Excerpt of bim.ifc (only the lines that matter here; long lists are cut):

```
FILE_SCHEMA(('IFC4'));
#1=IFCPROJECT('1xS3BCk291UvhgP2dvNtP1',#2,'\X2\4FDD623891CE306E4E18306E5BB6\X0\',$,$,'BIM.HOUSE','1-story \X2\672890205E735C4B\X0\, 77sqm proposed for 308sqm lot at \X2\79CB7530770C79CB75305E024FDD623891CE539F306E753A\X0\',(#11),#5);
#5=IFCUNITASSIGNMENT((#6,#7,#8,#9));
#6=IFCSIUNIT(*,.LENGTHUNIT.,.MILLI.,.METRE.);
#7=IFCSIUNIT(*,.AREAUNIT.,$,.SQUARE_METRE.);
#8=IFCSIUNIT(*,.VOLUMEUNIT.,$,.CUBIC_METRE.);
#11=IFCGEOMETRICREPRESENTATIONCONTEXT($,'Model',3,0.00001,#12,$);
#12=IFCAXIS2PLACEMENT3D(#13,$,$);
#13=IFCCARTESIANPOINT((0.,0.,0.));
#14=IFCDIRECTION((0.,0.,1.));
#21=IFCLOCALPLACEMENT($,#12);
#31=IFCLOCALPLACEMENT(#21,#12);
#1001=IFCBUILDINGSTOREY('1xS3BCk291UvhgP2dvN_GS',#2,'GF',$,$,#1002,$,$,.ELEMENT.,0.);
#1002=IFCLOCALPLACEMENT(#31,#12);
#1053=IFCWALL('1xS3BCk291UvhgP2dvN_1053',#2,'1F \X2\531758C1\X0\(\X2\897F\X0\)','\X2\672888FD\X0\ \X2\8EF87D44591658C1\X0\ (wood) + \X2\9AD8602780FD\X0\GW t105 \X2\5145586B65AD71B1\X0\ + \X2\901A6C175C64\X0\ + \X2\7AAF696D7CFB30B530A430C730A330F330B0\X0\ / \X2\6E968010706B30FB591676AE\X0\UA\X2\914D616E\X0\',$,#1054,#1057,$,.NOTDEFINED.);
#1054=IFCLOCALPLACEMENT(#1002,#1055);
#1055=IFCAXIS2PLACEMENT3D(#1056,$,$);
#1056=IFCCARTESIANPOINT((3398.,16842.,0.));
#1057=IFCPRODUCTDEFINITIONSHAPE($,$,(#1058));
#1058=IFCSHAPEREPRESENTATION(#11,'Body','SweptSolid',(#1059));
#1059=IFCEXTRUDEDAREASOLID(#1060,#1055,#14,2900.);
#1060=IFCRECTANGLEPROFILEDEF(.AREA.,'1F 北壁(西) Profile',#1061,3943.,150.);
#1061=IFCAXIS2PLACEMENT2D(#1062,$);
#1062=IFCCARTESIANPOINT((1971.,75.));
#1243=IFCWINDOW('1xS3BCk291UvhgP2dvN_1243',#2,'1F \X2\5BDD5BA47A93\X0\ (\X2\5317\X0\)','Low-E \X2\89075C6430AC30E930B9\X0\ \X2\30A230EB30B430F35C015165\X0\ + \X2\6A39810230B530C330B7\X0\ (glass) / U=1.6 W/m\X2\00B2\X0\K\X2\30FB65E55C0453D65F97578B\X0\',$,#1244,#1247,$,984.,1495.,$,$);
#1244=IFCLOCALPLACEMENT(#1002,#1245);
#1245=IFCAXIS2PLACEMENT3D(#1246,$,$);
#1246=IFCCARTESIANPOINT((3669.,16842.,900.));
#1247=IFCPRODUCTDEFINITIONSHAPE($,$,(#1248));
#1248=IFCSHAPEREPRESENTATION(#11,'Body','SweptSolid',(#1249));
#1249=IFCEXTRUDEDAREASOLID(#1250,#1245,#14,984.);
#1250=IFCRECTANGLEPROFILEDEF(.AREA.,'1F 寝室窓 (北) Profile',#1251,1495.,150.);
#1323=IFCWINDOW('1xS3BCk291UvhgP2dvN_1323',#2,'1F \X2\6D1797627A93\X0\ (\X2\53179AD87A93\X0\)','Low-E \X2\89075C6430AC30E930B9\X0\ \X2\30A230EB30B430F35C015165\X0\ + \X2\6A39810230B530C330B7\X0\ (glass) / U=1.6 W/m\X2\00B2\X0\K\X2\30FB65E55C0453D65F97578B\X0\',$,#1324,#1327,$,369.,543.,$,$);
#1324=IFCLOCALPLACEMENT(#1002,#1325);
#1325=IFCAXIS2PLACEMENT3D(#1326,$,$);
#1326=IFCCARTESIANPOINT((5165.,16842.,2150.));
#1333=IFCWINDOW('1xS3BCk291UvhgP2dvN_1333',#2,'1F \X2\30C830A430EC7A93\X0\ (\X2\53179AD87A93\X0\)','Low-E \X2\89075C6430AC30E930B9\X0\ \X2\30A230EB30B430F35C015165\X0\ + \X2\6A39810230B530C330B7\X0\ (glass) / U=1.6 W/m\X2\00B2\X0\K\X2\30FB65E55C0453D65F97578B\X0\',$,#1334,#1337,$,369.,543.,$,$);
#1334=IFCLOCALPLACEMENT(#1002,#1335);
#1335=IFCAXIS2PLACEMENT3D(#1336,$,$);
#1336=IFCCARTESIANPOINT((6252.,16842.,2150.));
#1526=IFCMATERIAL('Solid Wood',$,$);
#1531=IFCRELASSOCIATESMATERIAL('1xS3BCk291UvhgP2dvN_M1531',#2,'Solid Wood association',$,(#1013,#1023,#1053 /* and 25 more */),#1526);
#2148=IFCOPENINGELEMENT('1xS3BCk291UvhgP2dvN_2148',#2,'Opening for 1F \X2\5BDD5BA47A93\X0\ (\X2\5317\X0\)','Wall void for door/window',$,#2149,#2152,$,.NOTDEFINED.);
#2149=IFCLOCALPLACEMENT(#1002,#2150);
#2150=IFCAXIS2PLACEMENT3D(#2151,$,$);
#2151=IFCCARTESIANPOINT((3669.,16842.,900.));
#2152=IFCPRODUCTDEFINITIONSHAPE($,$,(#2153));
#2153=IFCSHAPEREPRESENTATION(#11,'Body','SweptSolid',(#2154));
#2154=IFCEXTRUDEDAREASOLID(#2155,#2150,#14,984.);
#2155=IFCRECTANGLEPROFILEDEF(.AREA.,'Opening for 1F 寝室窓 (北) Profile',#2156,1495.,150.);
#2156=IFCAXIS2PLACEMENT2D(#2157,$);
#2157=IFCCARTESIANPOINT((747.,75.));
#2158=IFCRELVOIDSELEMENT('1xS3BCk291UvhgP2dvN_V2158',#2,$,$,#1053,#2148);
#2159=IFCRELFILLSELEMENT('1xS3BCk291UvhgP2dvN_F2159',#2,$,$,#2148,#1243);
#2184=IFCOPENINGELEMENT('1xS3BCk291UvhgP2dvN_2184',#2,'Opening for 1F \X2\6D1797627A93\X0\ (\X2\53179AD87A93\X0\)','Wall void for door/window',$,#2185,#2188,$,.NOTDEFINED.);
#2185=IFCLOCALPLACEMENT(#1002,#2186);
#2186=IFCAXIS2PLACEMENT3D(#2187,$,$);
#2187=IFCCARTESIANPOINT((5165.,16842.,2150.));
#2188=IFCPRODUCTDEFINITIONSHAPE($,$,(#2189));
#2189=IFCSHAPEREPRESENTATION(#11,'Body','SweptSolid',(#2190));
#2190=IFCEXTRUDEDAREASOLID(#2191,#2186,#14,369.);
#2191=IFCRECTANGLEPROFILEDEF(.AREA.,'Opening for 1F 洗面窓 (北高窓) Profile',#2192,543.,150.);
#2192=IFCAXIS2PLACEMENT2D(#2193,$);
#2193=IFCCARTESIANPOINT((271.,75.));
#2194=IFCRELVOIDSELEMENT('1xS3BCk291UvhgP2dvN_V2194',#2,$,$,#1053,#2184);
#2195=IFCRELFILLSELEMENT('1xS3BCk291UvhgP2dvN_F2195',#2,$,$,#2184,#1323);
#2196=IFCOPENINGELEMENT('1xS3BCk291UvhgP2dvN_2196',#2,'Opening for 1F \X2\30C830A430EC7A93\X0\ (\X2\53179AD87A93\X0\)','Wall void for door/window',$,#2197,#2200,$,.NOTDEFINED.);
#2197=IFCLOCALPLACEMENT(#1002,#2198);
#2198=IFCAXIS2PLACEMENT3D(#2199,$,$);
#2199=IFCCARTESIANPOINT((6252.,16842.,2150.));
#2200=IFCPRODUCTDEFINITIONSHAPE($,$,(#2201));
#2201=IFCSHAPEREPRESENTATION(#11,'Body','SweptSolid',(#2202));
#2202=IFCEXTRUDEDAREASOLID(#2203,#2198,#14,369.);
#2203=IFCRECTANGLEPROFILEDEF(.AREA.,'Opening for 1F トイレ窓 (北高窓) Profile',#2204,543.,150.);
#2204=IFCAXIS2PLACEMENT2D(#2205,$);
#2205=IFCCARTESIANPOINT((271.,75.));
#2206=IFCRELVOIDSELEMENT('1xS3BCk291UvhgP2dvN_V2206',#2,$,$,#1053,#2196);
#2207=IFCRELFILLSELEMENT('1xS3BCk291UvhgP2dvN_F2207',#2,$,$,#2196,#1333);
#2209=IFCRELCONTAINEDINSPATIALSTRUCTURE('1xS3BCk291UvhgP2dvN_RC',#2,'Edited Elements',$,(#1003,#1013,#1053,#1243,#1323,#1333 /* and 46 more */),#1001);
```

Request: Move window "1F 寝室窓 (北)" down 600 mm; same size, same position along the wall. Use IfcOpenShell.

```python
import numpy as np
import ifcopenshell
import ifcopenshell.api.geometry
import ifcopenshell.util.placement
import ifcopenshell.util.unit

model = ifcopenshell.open("bim.ifc")
unit_scale = ifcopenshell.util.unit.calculate_unit_scale(model)

window = model.by_guid("1xS3BCk291UvhgP2dvN_1243")
opening = window.FillsVoids[0].RelatingOpeningElement
dz = -600.0

shift = np.array([0.0, 0.0, dz])
# The window is not placed relative to its opening, so move both.
for product in (opening, window):
    matrix = ifcopenshell.util.placement.get_local_placement(product.ObjectPlacement)
    matrix[:3, 3] += shift
    ifcopenshell.api.geometry.edit_object_placement(model, product=product, matrix=matrix, is_si=False)

print(f"moved by {dz * unit_scale:+.3f} m")

model.write("bim_rev.ifc")
```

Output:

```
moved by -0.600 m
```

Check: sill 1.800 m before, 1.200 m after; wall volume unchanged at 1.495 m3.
